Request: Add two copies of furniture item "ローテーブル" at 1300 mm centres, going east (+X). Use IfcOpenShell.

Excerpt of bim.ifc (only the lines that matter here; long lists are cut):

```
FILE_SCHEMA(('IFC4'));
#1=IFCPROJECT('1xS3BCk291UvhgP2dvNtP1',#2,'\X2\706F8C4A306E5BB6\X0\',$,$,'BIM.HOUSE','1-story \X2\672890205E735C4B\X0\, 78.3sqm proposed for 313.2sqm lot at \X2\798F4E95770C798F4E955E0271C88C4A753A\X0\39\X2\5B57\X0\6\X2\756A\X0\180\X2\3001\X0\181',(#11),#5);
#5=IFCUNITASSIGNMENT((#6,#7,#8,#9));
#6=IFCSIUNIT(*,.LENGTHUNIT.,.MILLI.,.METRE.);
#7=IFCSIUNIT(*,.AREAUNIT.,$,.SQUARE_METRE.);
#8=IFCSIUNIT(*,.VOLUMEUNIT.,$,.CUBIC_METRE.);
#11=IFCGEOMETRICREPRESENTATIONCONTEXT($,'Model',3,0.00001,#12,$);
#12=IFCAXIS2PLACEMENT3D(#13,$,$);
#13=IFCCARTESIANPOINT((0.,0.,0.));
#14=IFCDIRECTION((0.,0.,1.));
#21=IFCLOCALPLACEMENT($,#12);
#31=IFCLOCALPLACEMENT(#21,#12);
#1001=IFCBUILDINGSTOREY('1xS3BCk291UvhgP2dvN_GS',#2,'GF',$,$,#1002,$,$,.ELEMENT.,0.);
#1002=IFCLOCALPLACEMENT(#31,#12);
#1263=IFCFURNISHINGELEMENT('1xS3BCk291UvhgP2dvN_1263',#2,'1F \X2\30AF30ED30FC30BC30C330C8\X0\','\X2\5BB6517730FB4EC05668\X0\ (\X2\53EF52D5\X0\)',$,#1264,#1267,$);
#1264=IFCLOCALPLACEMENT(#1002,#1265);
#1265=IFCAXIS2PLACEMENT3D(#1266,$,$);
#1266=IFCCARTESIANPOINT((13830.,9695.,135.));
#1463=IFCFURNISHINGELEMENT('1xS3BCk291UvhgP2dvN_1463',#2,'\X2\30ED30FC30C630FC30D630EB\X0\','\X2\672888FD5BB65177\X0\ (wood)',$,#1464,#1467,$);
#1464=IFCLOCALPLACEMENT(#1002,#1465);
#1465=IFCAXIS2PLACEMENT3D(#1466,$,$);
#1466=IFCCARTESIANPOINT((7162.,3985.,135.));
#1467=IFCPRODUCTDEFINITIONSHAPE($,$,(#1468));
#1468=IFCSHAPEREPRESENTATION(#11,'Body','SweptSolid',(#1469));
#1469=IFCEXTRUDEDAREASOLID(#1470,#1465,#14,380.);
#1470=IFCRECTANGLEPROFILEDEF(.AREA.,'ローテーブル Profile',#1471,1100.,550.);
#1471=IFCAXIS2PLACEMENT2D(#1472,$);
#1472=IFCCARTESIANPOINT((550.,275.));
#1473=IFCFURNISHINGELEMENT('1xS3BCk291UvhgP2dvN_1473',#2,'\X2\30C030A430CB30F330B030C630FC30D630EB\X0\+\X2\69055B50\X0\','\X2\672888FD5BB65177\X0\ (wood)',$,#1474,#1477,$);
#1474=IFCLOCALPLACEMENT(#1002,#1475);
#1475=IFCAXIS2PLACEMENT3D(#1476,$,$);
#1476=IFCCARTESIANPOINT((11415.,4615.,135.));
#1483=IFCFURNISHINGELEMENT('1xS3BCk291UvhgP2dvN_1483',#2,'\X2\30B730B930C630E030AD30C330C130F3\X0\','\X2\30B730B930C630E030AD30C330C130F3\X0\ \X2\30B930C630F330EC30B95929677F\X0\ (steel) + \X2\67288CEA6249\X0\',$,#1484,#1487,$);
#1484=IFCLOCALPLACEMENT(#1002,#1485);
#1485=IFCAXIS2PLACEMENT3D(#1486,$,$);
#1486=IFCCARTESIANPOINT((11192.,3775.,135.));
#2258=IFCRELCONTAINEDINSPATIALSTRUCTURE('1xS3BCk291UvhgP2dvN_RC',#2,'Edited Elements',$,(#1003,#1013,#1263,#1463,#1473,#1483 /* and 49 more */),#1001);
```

```python
import numpy as np
import ifcopenshell
import ifcopenshell.api.geometry
import ifcopenshell.api.root
import ifcopenshell.util.element
import ifcopenshell.util.placement
import ifcopenshell.util.unit

model = ifcopenshell.open("bim.ifc")
unit_scale = ifcopenshell.util.unit.calculate_unit_scale(model)


def reuse_history(source, copy):
    """copy_class also copies each property set's owner history, people and application; keep the originals."""
    for rel in copy.IsDefinedBy:
        if rel.is_a("IfcRelDefinesByProperties") and (history := rel.RelatingPropertyDefinition.OwnerHistory):
            rel.RelatingPropertyDefinition.OwnerHistory = source.OwnerHistory
            ifcopenshell.util.element.remove_deep2(model, history)


source = model.by_id(1463)
base = ifcopenshell.util.placement.get_local_placement(source.ObjectPlacement)
step = np.array([1.0, 0.0, 0.0]) * 1.3 / unit_scale

for i in range(1, 3):
    copy = ifcopenshell.api.root.copy_class(model, product=source)
    copy.Representation = ifcopenshell.util.element.copy_deep(
        model, source.Representation, exclude=["IfcGeometricRepresentationContext", "IfcRepresentationMap"]
    )
    reuse_history(source, copy)
    matrix = base.copy()
    matrix[:3, 3] += i * step
    print("added at", matrix[:3, 3].round(3) + 0.0)
    ifcopenshell.api.geometry.edit_object_placement(model, product=copy, matrix=matrix, is_si=False)

model.write("bim_v2.ifc")
```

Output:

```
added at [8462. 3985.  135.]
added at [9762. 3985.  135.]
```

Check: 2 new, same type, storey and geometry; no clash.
